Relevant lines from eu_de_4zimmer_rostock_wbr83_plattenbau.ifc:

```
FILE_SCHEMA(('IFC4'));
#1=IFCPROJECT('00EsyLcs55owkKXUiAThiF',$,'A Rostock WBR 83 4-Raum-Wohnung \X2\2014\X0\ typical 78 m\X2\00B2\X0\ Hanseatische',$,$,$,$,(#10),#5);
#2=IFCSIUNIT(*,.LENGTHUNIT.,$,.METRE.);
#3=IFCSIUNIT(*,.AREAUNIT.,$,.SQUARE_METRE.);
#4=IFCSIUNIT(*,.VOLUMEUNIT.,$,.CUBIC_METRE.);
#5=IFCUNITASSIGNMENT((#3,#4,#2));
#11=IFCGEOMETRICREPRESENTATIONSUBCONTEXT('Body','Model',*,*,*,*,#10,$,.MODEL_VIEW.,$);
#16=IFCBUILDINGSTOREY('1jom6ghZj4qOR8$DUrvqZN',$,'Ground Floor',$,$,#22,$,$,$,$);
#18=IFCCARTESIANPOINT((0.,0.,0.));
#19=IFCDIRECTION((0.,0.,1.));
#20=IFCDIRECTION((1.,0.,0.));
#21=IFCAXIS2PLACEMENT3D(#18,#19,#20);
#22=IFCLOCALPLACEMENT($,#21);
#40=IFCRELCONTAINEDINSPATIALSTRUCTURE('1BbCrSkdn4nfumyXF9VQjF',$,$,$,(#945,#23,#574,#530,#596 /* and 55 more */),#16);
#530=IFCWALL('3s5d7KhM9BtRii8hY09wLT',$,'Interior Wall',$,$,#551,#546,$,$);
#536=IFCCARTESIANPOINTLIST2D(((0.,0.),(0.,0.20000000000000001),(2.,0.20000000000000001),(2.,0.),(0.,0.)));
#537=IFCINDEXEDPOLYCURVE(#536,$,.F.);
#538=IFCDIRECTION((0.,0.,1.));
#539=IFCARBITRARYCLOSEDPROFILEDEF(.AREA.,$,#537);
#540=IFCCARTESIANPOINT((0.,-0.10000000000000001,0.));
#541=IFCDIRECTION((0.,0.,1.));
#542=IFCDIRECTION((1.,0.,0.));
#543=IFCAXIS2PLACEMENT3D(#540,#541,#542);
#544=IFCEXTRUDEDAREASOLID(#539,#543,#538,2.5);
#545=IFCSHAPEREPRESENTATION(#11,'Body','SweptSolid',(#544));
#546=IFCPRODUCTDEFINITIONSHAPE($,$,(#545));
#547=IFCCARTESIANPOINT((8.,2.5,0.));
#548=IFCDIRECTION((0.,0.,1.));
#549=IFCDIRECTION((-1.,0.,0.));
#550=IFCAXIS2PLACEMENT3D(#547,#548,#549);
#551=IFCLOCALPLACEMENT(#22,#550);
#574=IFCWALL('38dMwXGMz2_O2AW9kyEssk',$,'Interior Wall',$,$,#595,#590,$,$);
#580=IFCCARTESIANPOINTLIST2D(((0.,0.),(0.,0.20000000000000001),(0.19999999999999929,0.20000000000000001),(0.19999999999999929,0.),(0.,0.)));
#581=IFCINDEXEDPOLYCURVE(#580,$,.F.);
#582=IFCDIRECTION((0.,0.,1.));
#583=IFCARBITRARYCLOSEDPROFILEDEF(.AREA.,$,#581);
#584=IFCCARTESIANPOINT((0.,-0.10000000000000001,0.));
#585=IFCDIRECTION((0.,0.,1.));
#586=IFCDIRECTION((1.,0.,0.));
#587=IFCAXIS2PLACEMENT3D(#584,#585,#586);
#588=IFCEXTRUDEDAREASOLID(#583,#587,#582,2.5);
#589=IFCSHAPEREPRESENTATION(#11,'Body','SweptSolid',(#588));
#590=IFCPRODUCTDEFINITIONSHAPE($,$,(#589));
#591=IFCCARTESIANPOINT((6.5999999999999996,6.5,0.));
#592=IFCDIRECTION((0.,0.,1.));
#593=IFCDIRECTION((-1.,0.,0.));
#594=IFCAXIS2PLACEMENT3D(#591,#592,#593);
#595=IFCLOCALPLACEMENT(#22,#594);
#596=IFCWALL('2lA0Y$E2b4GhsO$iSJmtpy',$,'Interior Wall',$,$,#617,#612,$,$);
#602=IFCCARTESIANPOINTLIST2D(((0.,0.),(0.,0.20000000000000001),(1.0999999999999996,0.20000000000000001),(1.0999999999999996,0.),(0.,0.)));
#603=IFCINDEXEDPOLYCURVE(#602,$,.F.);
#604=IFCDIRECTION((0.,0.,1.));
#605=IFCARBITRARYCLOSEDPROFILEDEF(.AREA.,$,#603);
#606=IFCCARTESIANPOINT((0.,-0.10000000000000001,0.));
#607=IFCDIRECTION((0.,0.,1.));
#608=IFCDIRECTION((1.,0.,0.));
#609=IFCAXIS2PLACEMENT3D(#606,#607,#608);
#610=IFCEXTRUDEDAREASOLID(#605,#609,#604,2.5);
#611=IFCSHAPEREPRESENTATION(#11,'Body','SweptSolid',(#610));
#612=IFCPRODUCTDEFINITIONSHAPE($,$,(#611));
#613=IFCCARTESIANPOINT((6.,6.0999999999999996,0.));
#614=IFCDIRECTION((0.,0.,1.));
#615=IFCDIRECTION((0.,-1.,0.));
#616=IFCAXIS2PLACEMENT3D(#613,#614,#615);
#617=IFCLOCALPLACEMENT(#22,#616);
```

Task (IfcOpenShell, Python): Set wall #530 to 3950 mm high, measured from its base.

```python
import ifcopenshell
import ifcopenshell.geom
import ifcopenshell.util.representation
import ifcopenshell.util.shape
import ifcopenshell.util.unit

model = ifcopenshell.open("eu_de_4zimmer_rostock_wbr83_plattenbau.ifc")
unit_scale = ifcopenshell.util.unit.calculate_unit_scale(model)
settings = ifcopenshell.geom.settings()


def volume(element):
    """Net volume in cubic metres, openings subtracted."""
    shape = ifcopenshell.geom.create_shape(settings, element)
    return ifcopenshell.util.shape.get_volume(shape.geometry)


wall = model.by_guid("3s5d7KhM9BtRii8hY09wLT")
before = volume(wall)

body = ifcopenshell.util.representation.get_representation(wall, "Model", "Body")
solid = body.Items[0]
old_height = solid.Depth
solid.Depth = 3.95 / unit_scale
after = volume(wall)

print(f"height {old_height:g} -> {solid.Depth:g}, volume {before:.3f} -> {after:.3f} m3")

model.write("eu_de_4zimmer_rostock_wbr83_plattenbau-out.ifc")
```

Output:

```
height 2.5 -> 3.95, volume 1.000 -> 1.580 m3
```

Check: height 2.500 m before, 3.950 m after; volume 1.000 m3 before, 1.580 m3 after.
